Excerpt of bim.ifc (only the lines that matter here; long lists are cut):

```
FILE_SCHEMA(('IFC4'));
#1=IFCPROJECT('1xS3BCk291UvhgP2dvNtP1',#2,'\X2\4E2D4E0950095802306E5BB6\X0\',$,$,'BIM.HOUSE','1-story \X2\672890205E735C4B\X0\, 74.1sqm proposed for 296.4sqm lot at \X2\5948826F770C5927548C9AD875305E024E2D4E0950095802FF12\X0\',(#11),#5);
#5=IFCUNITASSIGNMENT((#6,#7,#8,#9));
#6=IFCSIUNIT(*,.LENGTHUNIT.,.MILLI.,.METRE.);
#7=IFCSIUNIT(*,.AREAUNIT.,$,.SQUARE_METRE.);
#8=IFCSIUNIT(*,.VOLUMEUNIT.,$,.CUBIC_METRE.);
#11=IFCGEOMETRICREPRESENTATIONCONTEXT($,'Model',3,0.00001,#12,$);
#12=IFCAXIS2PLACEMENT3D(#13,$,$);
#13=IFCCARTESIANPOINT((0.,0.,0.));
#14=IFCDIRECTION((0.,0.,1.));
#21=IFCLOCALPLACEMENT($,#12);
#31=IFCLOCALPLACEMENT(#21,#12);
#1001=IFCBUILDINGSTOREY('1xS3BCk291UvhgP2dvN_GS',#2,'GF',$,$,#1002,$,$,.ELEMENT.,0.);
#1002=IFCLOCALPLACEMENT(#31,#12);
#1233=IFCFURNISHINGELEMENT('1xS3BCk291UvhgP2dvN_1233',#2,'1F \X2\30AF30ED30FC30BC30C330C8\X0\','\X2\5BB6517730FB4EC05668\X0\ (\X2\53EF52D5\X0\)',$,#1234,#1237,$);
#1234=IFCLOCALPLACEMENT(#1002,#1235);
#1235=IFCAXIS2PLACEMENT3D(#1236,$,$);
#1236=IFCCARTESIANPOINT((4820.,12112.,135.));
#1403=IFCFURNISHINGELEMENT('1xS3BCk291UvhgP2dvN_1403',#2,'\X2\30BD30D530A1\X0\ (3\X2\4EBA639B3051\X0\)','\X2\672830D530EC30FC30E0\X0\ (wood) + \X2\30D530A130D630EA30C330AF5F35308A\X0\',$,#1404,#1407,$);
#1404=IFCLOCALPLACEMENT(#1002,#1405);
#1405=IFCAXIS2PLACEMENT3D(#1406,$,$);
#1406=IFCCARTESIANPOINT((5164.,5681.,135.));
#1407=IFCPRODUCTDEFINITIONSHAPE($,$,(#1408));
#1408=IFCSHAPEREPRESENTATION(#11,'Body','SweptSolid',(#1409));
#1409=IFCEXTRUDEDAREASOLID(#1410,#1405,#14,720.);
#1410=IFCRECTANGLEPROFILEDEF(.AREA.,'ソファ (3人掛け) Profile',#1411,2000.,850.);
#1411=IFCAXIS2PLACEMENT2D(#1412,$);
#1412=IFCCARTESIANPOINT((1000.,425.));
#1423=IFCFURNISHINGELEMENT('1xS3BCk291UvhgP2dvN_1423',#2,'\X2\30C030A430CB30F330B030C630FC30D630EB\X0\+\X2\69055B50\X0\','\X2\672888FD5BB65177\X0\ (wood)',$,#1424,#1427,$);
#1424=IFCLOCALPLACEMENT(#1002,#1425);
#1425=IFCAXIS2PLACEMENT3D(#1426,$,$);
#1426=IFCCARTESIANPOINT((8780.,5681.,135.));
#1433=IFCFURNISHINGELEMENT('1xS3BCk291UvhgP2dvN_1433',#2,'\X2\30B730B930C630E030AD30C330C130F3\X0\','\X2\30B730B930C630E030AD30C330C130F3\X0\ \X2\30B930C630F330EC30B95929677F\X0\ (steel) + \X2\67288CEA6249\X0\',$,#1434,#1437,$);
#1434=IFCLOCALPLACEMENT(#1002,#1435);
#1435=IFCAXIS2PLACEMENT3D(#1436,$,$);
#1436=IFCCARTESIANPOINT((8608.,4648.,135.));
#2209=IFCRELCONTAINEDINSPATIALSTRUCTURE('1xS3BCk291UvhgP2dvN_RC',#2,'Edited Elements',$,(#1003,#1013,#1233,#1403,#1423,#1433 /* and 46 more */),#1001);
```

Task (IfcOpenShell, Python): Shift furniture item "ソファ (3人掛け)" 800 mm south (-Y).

```python
import ifcopenshell
import ifcopenshell.api.geometry
import ifcopenshell.util.placement
import ifcopenshell.util.unit

model = ifcopenshell.open("bim.ifc")
unit_scale = ifcopenshell.util.unit.calculate_unit_scale(model)

item = model.by_guid("1xS3BCk291UvhgP2dvN_1403")
matrix = ifcopenshell.util.placement.get_local_placement(item.ObjectPlacement)
matrix[1, 3] -= 0.8 / unit_scale
ifcopenshell.api.geometry.edit_object_placement(model, product=item, matrix=matrix, is_si=False)

print(ifcopenshell.util.placement.get_local_placement(item.ObjectPlacement).round(3) + 0.0)

model.write("bim_updated.ifc")
```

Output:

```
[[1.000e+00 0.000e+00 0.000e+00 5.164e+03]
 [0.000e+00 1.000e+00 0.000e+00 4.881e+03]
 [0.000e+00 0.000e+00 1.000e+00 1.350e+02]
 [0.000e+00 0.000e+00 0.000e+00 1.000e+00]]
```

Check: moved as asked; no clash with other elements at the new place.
